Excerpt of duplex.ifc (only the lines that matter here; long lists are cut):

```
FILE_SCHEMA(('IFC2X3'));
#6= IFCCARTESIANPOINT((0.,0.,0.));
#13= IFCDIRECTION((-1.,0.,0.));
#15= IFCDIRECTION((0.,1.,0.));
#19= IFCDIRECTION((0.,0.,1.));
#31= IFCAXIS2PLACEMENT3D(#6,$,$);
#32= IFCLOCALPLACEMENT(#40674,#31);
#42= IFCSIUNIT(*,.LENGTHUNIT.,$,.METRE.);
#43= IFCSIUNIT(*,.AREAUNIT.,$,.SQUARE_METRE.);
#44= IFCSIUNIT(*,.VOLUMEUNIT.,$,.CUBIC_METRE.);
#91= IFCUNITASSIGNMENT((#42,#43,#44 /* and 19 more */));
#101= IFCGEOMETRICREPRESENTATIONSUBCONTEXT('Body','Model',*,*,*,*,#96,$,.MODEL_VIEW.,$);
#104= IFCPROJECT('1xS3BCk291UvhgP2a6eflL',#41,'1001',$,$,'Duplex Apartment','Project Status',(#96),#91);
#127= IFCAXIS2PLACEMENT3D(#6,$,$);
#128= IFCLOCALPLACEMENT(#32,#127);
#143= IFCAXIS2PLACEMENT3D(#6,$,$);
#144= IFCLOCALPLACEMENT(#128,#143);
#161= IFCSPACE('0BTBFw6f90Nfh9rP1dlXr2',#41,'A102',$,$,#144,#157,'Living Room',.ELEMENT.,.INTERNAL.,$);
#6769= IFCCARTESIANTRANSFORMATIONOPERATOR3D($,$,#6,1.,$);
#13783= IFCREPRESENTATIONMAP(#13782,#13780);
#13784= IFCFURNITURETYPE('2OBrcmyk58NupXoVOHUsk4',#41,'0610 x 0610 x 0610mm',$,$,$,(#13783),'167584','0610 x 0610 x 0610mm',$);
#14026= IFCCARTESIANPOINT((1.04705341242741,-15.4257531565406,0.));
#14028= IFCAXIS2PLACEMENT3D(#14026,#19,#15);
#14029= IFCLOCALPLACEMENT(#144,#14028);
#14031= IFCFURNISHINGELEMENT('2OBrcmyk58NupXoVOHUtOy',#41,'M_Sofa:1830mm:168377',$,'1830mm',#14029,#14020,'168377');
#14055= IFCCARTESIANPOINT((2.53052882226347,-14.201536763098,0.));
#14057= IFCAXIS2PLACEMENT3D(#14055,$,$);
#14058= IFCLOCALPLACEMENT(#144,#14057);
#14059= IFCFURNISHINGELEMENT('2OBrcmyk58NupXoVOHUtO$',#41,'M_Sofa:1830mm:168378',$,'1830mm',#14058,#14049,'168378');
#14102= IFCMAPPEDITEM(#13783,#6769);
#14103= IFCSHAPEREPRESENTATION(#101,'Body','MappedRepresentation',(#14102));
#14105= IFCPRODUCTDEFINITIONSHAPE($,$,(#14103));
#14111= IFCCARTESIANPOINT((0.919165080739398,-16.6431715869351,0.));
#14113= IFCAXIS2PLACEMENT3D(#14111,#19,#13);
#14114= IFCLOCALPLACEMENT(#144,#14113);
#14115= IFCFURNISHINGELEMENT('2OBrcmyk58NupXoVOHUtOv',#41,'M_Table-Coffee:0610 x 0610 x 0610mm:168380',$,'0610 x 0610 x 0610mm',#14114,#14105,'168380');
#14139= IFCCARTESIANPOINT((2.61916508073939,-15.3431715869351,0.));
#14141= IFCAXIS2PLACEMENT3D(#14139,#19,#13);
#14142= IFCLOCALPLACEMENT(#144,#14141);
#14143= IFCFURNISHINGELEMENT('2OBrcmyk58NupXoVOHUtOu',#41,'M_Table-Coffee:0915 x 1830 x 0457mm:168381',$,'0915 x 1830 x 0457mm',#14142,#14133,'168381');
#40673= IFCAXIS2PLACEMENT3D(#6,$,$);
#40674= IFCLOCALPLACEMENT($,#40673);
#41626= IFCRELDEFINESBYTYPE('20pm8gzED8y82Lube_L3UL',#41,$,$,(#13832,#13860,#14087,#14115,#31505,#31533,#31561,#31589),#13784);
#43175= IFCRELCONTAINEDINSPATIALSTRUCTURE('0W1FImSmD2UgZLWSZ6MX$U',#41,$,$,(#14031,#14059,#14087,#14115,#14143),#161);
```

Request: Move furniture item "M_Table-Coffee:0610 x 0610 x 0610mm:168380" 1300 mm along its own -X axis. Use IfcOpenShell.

```python
import ifcopenshell
import ifcopenshell.api.geometry
import ifcopenshell.util.placement
import ifcopenshell.util.unit

model = ifcopenshell.open("duplex.ifc")
unit_scale = ifcopenshell.util.unit.calculate_unit_scale(model)

item = model.by_guid("2OBrcmyk58NupXoVOHUtOv")
matrix = ifcopenshell.util.placement.get_local_placement(item.ObjectPlacement)
matrix[:3, 3] -= matrix[:3, 0] * 1.3 / unit_scale
ifcopenshell.api.geometry.edit_object_placement(model, product=item, matrix=matrix, is_si=False)

print(ifcopenshell.util.placement.get_local_placement(item.ObjectPlacement).round(3) + 0.0)

model.write("duplex_edited.ifc")
```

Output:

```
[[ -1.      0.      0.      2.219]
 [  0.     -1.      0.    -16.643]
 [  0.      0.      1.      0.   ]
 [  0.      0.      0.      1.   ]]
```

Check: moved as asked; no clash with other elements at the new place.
